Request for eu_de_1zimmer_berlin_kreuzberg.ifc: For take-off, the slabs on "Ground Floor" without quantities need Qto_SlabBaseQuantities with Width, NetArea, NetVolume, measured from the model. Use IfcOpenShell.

First a look at what the model holds.

```python
import ifcopenshell
import ifcopenshell.util.element
import ifcopenshell.util.unit

model = ifcopenshell.open("eu_de_1zimmer_berlin_kreuzberg.ifc")
print(model.schema)
for unit_type in ("LENGTHUNIT", "AREAUNIT", "VOLUMEUNIT"):
    print(unit_type, ifcopenshell.util.unit.calculate_unit_scale(model, unit_type))
storey = next(s for s in model.by_type("IfcBuildingStorey") if s.Name == "Ground Floor")
slabs = [e for e in ifcopenshell.util.element.get_decomposition(storey) if e.is_a("IfcSlab")]
for e in sorted(slabs, key=lambda e: e.id()):
    print(e.id(), e.is_a(), e.Name, list(ifcopenshell.util.element.get_psets(e, qtos_only=True)), sep=" | ")
```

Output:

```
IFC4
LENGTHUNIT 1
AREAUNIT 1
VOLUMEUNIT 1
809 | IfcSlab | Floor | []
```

```python
import ifcopenshell
import ifcopenshell.api.pset
import ifcopenshell.geom
import ifcopenshell.util.element
import ifcopenshell.util.shape
import ifcopenshell.util.unit

model = ifcopenshell.open("eu_de_1zimmer_berlin_kreuzberg.ifc")
unit_scale = ifcopenshell.util.unit.calculate_unit_scale(model)
area_scale = ifcopenshell.util.unit.calculate_unit_scale(model, "AREAUNIT")
volume_scale = ifcopenshell.util.unit.calculate_unit_scale(model, "VOLUMEUNIT")
settings = ifcopenshell.geom.settings()

storey = next(s for s in model.by_type("IfcBuildingStorey") if s.Name == "Ground Floor")
slabs = [e for e in ifcopenshell.util.element.get_decomposition(storey) if e.is_a("IfcSlab")]

for e in sorted(slabs, key=lambda e: e.id()):
    if ifcopenshell.util.element.get_psets(e, qtos_only=True, should_inherit=False):
        continue
    # Geometry comes back in metres, in the element's own axes.
    shape = ifcopenshell.geom.create_shape(settings, e)
    values = {
        "Width": ifcopenshell.util.shape.get_z(shape.geometry) / unit_scale,
        "NetArea": ifcopenshell.util.shape.get_footprint_area(shape.geometry) / area_scale,
        "NetVolume": ifcopenshell.util.shape.get_volume(shape.geometry) / volume_scale,
    }
    qto = ifcopenshell.api.pset.add_qto(model, product=e, name="Qto_SlabBaseQuantities")
    ifcopenshell.api.pset.edit_qto(model, qto=qto, properties=values)
    print(e.id(), {k: round(v, 3) for k, v in values.items()})

model.write("eu_de_1zimmer_berlin_kreuzberg_v2.ifc")
```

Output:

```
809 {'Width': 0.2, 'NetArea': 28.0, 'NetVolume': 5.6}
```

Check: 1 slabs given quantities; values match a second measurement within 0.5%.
